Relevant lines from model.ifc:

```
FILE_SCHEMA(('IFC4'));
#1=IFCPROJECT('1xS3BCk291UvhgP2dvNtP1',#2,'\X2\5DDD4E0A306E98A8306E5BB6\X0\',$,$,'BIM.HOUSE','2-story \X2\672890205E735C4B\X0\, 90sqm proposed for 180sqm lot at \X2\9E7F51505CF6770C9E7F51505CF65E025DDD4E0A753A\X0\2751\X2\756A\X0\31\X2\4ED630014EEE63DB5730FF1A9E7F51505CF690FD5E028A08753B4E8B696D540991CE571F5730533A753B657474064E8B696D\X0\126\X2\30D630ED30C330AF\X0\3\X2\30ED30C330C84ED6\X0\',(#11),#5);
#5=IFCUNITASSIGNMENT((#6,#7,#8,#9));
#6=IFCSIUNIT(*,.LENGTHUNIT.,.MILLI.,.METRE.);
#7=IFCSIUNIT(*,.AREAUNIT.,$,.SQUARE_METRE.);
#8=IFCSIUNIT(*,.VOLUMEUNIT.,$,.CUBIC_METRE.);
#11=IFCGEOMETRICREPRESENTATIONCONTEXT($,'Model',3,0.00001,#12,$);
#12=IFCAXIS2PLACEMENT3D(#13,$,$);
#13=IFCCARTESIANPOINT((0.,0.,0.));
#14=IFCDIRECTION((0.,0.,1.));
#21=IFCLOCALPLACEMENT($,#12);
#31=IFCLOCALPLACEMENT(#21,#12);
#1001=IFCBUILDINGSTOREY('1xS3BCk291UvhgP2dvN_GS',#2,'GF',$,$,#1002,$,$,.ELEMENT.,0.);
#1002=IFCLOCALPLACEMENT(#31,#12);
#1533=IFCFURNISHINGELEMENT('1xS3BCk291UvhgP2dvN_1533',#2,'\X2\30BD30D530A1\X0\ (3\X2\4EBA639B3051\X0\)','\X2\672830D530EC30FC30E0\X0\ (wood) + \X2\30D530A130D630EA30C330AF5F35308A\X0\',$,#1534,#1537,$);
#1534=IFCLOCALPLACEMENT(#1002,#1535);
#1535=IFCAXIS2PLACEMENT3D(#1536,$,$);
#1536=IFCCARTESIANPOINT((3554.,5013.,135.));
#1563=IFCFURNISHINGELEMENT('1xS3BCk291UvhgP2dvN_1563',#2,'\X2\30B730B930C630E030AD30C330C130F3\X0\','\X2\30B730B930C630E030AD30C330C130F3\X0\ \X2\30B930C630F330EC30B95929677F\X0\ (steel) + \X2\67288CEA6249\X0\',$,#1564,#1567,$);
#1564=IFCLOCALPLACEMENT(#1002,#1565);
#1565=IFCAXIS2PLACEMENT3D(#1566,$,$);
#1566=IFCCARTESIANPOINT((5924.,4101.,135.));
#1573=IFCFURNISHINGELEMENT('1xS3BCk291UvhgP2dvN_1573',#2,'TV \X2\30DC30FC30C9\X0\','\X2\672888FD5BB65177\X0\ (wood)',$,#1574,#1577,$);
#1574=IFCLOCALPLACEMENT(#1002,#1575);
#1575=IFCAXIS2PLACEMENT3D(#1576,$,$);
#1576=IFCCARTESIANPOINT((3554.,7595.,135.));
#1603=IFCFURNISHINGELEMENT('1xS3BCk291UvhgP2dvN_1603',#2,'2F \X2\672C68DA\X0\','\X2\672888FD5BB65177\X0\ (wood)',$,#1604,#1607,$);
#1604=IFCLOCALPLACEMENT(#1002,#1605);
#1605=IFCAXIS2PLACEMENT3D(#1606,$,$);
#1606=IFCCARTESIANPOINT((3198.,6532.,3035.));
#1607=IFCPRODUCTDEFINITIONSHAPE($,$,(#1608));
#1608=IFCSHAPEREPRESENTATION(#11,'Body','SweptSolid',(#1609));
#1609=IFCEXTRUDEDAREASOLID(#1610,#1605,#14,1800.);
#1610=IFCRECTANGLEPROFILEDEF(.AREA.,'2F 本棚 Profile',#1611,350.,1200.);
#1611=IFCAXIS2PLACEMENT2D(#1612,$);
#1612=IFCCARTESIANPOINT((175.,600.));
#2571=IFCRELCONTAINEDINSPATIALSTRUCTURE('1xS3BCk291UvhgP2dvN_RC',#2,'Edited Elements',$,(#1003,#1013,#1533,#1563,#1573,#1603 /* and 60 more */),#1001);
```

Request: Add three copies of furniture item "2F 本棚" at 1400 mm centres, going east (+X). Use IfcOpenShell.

```python
import numpy as np
import ifcopenshell
import ifcopenshell.api.geometry
import ifcopenshell.api.root
import ifcopenshell.util.element
import ifcopenshell.util.placement

model = ifcopenshell.open("model.ifc")


def reuse_history(source, copy):
    """copy_class also copies each property set's owner history, people and application; keep the originals."""
    for rel in copy.IsDefinedBy:
        if rel.is_a("IfcRelDefinesByProperties") and (history := rel.RelatingPropertyDefinition.OwnerHistory):
            rel.RelatingPropertyDefinition.OwnerHistory = source.OwnerHistory
            ifcopenshell.util.element.remove_deep2(model, history)


source = model.by_id(1603)
base = ifcopenshell.util.placement.get_local_placement(source.ObjectPlacement)
step = np.array([1.0, 0.0, 0.0]) * 1400.0

for i in range(1, 4):
    copy = ifcopenshell.api.root.copy_class(model, product=source)
    copy.Representation = ifcopenshell.util.element.copy_deep(
        model, source.Representation, exclude=["IfcGeometricRepresentationContext", "IfcRepresentationMap"]
    )
    reuse_history(source, copy)
    matrix = base.copy()
    matrix[:3, 3] += i * step
    print("added at", matrix[:3, 3].round(3) + 0.0)
    ifcopenshell.api.geometry.edit_object_placement(model, product=copy, matrix=matrix, is_si=False)

model.write("model-out.ifc")
```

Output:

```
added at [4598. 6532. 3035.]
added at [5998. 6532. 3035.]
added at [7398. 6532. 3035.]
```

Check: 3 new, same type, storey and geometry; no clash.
